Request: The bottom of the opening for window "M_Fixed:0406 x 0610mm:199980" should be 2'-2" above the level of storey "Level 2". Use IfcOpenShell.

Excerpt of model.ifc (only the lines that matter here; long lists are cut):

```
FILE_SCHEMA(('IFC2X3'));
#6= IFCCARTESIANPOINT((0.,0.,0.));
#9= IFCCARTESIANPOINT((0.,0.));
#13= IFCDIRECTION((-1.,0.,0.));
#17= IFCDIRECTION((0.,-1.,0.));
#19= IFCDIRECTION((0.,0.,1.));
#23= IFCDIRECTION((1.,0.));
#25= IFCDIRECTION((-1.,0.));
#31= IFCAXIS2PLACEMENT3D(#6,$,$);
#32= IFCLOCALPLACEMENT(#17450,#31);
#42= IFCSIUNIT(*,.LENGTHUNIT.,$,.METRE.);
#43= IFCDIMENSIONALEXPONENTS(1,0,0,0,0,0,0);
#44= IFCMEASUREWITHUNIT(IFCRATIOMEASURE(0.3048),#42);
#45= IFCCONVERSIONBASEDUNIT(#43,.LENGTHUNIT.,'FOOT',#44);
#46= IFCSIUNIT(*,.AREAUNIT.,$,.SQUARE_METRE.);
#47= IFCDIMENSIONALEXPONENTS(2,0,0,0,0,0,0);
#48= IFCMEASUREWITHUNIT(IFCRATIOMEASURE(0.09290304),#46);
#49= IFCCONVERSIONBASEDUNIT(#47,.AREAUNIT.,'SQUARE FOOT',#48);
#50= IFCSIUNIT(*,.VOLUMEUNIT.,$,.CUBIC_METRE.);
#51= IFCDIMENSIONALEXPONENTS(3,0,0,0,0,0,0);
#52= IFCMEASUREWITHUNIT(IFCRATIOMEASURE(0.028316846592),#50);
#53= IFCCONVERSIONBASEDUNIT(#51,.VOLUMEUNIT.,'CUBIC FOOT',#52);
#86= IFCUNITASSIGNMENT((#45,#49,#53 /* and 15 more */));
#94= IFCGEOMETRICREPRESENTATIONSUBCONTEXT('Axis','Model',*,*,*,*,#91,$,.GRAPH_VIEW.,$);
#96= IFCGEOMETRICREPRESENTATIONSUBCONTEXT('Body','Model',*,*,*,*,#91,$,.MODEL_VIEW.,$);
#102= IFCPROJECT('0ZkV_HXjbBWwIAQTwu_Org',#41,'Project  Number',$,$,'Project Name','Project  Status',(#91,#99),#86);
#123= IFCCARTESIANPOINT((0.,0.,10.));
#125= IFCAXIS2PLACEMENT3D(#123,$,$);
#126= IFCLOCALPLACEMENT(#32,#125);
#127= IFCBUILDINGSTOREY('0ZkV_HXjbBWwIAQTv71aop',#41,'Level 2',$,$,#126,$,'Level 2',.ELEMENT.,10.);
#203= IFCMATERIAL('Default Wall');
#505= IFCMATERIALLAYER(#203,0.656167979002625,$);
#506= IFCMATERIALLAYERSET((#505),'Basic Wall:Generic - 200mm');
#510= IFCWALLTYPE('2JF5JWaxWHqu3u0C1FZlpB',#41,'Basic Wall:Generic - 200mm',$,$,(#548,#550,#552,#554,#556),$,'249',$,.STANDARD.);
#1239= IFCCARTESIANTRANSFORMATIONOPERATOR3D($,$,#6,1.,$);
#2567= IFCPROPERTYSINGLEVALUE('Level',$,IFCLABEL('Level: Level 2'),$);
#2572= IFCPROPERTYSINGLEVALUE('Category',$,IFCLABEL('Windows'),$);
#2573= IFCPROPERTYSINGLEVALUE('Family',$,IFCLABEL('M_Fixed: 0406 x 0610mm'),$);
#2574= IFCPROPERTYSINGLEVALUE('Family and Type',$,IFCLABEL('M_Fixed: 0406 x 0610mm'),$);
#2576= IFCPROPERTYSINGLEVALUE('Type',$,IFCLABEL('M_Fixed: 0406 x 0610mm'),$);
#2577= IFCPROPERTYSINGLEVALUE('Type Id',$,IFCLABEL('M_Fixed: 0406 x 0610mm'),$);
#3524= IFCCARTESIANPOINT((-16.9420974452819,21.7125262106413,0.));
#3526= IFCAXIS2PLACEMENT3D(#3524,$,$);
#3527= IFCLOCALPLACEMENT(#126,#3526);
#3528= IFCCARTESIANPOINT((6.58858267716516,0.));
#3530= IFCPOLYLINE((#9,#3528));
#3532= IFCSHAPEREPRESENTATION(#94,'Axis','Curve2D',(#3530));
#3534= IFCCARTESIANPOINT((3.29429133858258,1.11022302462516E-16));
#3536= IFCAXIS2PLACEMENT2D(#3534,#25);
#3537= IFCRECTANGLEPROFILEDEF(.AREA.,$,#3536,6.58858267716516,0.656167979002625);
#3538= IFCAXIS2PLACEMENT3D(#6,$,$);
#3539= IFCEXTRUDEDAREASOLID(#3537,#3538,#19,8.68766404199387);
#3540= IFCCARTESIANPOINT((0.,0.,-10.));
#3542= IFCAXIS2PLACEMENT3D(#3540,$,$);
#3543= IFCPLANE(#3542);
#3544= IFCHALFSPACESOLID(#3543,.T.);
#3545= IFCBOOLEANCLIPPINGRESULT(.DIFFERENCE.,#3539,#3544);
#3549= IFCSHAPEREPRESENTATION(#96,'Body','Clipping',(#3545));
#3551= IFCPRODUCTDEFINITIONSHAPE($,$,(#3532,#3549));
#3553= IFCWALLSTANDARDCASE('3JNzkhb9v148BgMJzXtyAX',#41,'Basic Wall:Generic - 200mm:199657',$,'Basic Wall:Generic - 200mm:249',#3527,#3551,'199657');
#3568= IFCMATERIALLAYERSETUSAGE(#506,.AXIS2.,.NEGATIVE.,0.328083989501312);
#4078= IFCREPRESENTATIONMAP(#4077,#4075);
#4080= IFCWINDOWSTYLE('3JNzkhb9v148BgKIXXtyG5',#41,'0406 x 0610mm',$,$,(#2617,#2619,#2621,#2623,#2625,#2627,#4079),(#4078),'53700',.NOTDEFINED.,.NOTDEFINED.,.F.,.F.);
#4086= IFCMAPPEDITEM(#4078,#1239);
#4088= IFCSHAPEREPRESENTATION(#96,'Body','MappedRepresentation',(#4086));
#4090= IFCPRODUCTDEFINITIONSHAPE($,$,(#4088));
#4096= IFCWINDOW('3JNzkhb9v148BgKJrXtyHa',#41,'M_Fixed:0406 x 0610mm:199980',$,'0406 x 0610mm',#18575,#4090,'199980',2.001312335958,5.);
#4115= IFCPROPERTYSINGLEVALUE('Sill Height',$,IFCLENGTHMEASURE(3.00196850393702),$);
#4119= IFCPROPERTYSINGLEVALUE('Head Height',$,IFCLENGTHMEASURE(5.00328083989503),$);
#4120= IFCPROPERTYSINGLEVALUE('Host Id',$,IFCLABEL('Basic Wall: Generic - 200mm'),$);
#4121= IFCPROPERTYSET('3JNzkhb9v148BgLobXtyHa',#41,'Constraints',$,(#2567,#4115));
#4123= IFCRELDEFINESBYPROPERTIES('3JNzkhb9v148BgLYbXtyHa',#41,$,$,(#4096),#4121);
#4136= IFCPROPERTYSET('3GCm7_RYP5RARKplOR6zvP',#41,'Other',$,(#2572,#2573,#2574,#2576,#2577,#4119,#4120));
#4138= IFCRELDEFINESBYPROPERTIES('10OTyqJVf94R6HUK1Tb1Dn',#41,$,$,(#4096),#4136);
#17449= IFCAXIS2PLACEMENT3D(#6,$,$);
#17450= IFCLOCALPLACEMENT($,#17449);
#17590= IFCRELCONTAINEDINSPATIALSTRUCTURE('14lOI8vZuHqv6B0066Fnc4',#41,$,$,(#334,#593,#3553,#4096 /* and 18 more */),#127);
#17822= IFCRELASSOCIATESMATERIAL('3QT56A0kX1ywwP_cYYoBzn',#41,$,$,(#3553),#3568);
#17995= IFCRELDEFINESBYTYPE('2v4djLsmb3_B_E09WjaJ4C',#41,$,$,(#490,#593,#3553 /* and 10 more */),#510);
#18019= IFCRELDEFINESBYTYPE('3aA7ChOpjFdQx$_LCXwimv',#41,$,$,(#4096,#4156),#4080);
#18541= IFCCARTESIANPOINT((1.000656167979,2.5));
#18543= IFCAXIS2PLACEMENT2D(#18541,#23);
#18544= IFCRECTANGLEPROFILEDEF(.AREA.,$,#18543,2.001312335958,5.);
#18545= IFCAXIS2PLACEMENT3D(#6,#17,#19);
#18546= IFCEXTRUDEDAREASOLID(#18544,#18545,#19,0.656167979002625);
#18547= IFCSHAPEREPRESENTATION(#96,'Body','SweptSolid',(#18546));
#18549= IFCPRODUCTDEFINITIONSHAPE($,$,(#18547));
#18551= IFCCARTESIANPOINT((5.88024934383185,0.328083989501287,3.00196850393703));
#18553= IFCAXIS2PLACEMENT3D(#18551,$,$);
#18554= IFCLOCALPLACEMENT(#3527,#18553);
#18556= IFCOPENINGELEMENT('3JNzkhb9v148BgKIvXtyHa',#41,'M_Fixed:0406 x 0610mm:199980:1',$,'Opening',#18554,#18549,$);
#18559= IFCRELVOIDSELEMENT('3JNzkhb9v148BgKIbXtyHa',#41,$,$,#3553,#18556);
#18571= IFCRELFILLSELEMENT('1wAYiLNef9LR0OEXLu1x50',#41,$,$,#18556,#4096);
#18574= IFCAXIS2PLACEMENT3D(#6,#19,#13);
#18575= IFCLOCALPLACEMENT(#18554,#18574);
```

```python
import numpy as np
import ifcopenshell
import ifcopenshell.api.geometry
import ifcopenshell.api.pset
import ifcopenshell.geom
import ifcopenshell.util.element
import ifcopenshell.util.placement
import ifcopenshell.util.shape
import ifcopenshell.util.unit

model = ifcopenshell.open("model.ifc")
unit_scale = ifcopenshell.util.unit.calculate_unit_scale(model)

window = model.by_guid("3JNzkhb9v148BgKJrXtyHa")
opening = window.FillsVoids[0].RelatingOpeningElement
storey = ifcopenshell.util.element.get_container(window, ifc_class="IfcBuildingStorey")
level = ifcopenshell.util.placement.get_local_placement(storey.ObjectPlacement)[2, 3]

# The opening's origin need not be at the sill, so measure its lowest point.
shape = ifcopenshell.geom.create_shape(ifcopenshell.geom.settings(), opening)
bottom = ifcopenshell.util.shape.get_shape_bottom_elevation(shape, shape.geometry) / unit_scale
dz = level + 26 * 0.0254 / unit_scale - bottom

shift = np.array([0.0, 0.0, dz])
# The window is placed relative to its opening, so it follows when the opening moves.
matrix = ifcopenshell.util.placement.get_local_placement(opening.ObjectPlacement)
matrix[:3, 3] += shift
ifcopenshell.api.geometry.edit_object_placement(
    model, product=opening, matrix=matrix, is_si=False, should_transform_children=True
)

# Keep the stored heights in step.
pset = model.by_id(ifcopenshell.util.element.get_pset(window, "Constraints", should_inherit=False)["id"])
ifcopenshell.api.pset.edit_pset(model, pset=pset, properties={
    "Sill Height": model.create_entity("IfcLengthMeasure", ifcopenshell.util.element.get_pset(window, "Constraints", "Sill Height") + dz),
})
pset = model.by_id(ifcopenshell.util.element.get_pset(window, "Other", should_inherit=False)["id"])
ifcopenshell.api.pset.edit_pset(model, pset=pset, properties={
    "Head Height": model.create_entity("IfcLengthMeasure", ifcopenshell.util.element.get_pset(window, "Other", "Head Height") + dz),
})

print(f"moved by {dz * unit_scale:+.3f} m")

model.write("model_rev.ifc")
```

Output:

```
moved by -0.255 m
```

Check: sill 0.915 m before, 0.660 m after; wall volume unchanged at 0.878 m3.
